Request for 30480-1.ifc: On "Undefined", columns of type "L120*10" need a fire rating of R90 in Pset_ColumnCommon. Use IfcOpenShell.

First a look at what the model holds.

```python
import ifcopenshell
import ifcopenshell.util.element

model = ifcopenshell.open("30480-1.ifc")
print(model.schema)
storey = next(s for s in model.by_type("IfcBuildingStorey") if s.Name == "Undefined")
columns = [e for e in ifcopenshell.util.element.get_decomposition(storey) if e.is_a("IfcColumn")]
seen = {}
for e in columns:
    element_type = ifcopenshell.util.element.get_type(e)
    key = (element_type.Name if element_type != e and element_type else None, ifcopenshell.util.element.get_pset(e, "Pset_ColumnCommon", "FireRating"))
    seen[key] = seen.get(key, 0) + 1
for (name, value), count in sorted(seen.items(), key=str):
    print(count, "x", name, "|", value)
```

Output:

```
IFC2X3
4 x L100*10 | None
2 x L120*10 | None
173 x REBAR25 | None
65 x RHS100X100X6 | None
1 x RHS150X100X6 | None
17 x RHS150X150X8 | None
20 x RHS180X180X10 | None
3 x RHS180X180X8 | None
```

```python
import ifcopenshell
import ifcopenshell.api.pset
import ifcopenshell.util.element

model = ifcopenshell.open("30480-1.ifc")

storey = next(s for s in model.by_type("IfcBuildingStorey") if s.Name == "Undefined")
columns = [e for e in ifcopenshell.util.element.get_decomposition(storey) if e.is_a("IfcColumn")]

count = 0
for e in columns:
    element_type = ifcopenshell.util.element.get_type(e)
    if element_type in (None, e) or element_type.Name != "L120*10":
        continue
    # add_pset returns the element's existing set when there is one.
    pset = ifcopenshell.api.pset.add_pset(model, product=e, name="Pset_ColumnCommon")
    ifcopenshell.api.pset.edit_pset(model, pset=pset, properties={"FireRating": "R90"})
    count += 1

print(count, "columns updated")

model.write("30480-1-out.ifc")
```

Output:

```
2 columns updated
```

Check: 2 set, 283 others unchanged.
